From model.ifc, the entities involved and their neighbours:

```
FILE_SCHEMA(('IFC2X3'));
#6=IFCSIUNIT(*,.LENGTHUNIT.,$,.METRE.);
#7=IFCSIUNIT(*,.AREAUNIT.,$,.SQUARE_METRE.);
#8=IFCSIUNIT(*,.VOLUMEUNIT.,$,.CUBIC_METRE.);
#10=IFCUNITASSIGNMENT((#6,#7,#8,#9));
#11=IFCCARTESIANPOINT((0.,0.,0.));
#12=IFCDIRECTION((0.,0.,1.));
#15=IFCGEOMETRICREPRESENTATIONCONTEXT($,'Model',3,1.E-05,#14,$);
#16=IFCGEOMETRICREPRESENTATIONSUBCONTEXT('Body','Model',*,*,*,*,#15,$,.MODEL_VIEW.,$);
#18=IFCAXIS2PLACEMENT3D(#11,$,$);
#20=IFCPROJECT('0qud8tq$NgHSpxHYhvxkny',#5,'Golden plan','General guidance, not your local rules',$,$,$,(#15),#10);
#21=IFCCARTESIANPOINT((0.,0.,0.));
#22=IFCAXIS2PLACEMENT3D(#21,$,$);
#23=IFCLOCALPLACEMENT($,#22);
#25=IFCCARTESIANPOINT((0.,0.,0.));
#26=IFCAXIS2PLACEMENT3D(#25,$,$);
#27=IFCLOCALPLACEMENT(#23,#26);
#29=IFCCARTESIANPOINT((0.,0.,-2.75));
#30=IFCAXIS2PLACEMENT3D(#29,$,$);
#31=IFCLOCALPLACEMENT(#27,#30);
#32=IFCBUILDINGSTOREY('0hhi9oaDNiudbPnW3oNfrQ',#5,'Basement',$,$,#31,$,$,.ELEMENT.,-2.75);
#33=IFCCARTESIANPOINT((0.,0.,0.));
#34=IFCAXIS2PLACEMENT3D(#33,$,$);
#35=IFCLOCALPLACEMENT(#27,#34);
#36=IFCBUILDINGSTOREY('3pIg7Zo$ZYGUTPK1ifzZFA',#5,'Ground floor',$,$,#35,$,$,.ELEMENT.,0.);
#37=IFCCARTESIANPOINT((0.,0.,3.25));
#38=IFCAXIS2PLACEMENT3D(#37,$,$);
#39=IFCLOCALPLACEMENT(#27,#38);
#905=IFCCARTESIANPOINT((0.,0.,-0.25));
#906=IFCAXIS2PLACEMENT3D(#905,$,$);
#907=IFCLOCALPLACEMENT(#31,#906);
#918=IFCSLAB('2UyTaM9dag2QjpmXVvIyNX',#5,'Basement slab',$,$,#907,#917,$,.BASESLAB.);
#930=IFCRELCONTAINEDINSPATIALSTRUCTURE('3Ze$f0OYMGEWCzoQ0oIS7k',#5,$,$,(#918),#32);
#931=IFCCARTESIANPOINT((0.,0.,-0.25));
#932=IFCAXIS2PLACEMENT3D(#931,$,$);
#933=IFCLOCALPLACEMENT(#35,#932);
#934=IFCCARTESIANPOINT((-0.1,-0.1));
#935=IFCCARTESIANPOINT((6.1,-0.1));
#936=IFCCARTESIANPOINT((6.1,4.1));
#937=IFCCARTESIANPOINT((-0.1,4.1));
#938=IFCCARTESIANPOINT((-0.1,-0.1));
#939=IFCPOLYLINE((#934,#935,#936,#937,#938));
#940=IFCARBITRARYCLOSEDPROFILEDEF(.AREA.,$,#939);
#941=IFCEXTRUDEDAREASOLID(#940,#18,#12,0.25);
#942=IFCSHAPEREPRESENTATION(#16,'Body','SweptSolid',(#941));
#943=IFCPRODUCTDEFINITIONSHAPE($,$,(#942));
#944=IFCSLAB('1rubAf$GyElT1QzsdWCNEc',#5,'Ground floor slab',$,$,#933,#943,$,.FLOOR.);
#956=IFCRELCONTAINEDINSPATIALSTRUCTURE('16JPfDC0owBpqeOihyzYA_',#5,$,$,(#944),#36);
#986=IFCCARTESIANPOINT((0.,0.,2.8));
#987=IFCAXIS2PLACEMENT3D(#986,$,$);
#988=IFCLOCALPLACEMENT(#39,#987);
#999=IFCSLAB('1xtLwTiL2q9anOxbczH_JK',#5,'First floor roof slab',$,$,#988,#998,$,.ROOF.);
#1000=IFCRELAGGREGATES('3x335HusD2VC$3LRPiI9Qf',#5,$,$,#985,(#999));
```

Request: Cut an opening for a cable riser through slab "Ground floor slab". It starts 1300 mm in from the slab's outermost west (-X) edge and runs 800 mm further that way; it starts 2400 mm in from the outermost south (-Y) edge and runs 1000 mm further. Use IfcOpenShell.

```python
import numpy as np
import ifcopenshell
import ifcopenshell.api.feature
import ifcopenshell.api.geometry
import ifcopenshell.api.root
import ifcopenshell.geom
import ifcopenshell.util.placement
import ifcopenshell.util.representation
import ifcopenshell.util.shape
import ifcopenshell.util.unit

model = ifcopenshell.open("model.ifc")
unit_scale = ifcopenshell.util.unit.calculate_unit_scale(model)
settings = ifcopenshell.geom.settings()


def volume(element):
    """Net volume in cubic metres, openings subtracted."""
    shape = ifcopenshell.geom.create_shape(settings, element)
    return ifcopenshell.util.shape.get_volume(shape.geometry)


slab = model.by_guid("1rubAf$GyElT1QzsdWCNEc")
before = volume(slab)

# Extent in the slab's own axes, in metres. The edges named are its -X and -Y sides.
slab_shape = ifcopenshell.geom.create_shape(settings, slab)
vertices = ifcopenshell.util.shape.get_vertices(slab_shape.geometry)
x_min, y_min, bottom = vertices.min(axis=0)
top = vertices[:, 2].max()

opening = ifcopenshell.api.root.create_entity(model, ifc_class="IfcOpeningElement", name="Cable riser opening")
context = ifcopenshell.util.representation.get_context(model, "Model", "Body", "MODEL_VIEW")
width, depth = 0.8, 1
outline = [(0.0, 0.0), (width, 0.0), (width, depth), (0.0, depth), (0.0, 0.0)]
# Overshoot both faces by 50 mm so the cut is clean.
shape = ifcopenshell.api.geometry.add_slab_representation(
    model, context=context, depth=top - bottom + 0.1, polyline=outline
)
ifcopenshell.api.geometry.assign_representation(model, product=opening, representation=shape)

matrix = ifcopenshell.util.placement.get_local_placement(slab.ObjectPlacement)
matrix[:, 3] = matrix @ np.append(np.array([x_min + 1.3, y_min + 2.4, bottom - 0.05]) / unit_scale, 1.0)
ifcopenshell.api.geometry.edit_object_placement(model, product=opening, matrix=matrix, is_si=False)
ifcopenshell.api.feature.add_feature(model, feature=opening, element=slab)

after = volume(slab)

print(f"slab volume {before:.3f} -> {after:.3f} m3")

model.write("model-out.ifc")
```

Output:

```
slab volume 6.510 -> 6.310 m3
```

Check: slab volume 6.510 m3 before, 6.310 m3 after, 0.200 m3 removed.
